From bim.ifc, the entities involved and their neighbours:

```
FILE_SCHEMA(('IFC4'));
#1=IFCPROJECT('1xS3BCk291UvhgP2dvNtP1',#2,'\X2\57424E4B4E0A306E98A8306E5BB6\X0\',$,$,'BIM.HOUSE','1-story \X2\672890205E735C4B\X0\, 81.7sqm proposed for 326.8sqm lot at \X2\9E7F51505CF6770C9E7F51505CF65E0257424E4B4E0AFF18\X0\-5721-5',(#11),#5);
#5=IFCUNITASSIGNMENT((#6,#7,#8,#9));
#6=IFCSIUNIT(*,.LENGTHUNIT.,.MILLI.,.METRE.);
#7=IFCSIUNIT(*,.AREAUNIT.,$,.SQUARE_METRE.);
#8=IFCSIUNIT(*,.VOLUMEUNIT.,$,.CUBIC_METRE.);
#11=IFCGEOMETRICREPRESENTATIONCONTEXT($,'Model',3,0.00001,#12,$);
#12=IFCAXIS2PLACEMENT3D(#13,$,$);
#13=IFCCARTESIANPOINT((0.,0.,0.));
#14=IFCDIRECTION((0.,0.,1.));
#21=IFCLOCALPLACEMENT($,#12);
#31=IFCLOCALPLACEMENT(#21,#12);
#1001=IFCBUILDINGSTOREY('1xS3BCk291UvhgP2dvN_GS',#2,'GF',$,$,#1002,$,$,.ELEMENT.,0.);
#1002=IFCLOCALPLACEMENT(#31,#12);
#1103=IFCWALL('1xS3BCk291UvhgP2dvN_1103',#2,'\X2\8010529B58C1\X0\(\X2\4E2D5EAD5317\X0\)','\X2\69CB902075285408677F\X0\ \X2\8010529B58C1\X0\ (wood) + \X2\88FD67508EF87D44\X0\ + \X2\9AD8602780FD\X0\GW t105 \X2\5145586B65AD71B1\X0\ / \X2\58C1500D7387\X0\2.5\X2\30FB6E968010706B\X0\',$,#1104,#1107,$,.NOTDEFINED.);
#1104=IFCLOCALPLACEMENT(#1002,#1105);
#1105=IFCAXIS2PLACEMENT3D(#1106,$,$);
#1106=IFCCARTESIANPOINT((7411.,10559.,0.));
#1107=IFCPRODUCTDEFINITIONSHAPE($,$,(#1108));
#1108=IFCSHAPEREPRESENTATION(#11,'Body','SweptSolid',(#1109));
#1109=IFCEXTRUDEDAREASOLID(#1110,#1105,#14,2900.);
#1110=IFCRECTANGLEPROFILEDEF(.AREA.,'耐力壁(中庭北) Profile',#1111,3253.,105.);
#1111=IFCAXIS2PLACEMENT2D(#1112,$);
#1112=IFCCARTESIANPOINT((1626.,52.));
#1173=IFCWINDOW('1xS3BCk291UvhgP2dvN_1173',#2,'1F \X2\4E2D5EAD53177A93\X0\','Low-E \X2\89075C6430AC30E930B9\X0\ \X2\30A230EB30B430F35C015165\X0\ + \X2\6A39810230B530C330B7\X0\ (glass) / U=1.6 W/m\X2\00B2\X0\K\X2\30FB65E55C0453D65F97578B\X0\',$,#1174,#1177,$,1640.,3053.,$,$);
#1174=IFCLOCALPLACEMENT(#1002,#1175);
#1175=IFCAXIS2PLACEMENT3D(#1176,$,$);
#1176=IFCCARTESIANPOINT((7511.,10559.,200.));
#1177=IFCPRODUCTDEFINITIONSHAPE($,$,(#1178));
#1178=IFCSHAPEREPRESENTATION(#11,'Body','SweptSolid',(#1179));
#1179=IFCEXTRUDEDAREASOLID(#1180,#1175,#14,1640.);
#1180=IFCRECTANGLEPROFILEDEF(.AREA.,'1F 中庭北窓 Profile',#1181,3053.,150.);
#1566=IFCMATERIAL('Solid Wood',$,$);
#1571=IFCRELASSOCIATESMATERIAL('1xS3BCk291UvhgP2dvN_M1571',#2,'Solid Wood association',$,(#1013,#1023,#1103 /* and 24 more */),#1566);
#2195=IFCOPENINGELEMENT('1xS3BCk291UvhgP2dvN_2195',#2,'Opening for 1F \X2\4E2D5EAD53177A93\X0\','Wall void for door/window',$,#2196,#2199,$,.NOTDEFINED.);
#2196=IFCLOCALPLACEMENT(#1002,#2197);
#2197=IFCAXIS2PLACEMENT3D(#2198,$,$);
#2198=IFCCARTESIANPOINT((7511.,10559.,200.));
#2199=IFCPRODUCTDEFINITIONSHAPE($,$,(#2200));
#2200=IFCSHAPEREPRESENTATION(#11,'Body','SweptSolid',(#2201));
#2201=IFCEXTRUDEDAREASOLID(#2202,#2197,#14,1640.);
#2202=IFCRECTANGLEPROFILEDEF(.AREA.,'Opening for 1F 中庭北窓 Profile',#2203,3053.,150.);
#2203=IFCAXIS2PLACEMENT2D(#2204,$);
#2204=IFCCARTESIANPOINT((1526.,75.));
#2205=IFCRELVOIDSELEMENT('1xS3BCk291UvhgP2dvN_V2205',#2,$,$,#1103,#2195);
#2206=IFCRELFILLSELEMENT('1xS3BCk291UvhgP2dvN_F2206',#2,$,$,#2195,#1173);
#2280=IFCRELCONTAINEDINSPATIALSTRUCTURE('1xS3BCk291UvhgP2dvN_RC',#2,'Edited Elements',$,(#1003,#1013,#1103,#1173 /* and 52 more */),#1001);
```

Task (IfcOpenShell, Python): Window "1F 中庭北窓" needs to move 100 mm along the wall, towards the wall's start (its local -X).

```python
import ifcopenshell
import ifcopenshell.api.geometry
import ifcopenshell.util.placement
import ifcopenshell.util.unit

model = ifcopenshell.open("bim.ifc")
unit_scale = ifcopenshell.util.unit.calculate_unit_scale(model)

window = model.by_id(1173)
opening = window.FillsVoids[0].RelatingOpeningElement
wall = opening.VoidsElements[0].RelatingBuildingElement

wall_matrix = ifcopenshell.util.placement.get_local_placement(wall.ObjectPlacement)
shift = wall_matrix[:3, 0] * -0.1 / unit_scale
before = ifcopenshell.util.placement.get_local_placement(window.ObjectPlacement)[:3, 3].copy()

# The window is not placed relative to its opening, so move both.
for product in (opening, window):
    matrix = ifcopenshell.util.placement.get_local_placement(product.ObjectPlacement)
    matrix[:3, 3] += shift
    ifcopenshell.api.geometry.edit_object_placement(model, product=product, matrix=matrix, is_si=False)

after = ifcopenshell.util.placement.get_local_placement(window.ObjectPlacement)[:3, 3]
print("window moved by", (after - before).round(3) + 0.0)

model.write("bim_v2.ifc")
```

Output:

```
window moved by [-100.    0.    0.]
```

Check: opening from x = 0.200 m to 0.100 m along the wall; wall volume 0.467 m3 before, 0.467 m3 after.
